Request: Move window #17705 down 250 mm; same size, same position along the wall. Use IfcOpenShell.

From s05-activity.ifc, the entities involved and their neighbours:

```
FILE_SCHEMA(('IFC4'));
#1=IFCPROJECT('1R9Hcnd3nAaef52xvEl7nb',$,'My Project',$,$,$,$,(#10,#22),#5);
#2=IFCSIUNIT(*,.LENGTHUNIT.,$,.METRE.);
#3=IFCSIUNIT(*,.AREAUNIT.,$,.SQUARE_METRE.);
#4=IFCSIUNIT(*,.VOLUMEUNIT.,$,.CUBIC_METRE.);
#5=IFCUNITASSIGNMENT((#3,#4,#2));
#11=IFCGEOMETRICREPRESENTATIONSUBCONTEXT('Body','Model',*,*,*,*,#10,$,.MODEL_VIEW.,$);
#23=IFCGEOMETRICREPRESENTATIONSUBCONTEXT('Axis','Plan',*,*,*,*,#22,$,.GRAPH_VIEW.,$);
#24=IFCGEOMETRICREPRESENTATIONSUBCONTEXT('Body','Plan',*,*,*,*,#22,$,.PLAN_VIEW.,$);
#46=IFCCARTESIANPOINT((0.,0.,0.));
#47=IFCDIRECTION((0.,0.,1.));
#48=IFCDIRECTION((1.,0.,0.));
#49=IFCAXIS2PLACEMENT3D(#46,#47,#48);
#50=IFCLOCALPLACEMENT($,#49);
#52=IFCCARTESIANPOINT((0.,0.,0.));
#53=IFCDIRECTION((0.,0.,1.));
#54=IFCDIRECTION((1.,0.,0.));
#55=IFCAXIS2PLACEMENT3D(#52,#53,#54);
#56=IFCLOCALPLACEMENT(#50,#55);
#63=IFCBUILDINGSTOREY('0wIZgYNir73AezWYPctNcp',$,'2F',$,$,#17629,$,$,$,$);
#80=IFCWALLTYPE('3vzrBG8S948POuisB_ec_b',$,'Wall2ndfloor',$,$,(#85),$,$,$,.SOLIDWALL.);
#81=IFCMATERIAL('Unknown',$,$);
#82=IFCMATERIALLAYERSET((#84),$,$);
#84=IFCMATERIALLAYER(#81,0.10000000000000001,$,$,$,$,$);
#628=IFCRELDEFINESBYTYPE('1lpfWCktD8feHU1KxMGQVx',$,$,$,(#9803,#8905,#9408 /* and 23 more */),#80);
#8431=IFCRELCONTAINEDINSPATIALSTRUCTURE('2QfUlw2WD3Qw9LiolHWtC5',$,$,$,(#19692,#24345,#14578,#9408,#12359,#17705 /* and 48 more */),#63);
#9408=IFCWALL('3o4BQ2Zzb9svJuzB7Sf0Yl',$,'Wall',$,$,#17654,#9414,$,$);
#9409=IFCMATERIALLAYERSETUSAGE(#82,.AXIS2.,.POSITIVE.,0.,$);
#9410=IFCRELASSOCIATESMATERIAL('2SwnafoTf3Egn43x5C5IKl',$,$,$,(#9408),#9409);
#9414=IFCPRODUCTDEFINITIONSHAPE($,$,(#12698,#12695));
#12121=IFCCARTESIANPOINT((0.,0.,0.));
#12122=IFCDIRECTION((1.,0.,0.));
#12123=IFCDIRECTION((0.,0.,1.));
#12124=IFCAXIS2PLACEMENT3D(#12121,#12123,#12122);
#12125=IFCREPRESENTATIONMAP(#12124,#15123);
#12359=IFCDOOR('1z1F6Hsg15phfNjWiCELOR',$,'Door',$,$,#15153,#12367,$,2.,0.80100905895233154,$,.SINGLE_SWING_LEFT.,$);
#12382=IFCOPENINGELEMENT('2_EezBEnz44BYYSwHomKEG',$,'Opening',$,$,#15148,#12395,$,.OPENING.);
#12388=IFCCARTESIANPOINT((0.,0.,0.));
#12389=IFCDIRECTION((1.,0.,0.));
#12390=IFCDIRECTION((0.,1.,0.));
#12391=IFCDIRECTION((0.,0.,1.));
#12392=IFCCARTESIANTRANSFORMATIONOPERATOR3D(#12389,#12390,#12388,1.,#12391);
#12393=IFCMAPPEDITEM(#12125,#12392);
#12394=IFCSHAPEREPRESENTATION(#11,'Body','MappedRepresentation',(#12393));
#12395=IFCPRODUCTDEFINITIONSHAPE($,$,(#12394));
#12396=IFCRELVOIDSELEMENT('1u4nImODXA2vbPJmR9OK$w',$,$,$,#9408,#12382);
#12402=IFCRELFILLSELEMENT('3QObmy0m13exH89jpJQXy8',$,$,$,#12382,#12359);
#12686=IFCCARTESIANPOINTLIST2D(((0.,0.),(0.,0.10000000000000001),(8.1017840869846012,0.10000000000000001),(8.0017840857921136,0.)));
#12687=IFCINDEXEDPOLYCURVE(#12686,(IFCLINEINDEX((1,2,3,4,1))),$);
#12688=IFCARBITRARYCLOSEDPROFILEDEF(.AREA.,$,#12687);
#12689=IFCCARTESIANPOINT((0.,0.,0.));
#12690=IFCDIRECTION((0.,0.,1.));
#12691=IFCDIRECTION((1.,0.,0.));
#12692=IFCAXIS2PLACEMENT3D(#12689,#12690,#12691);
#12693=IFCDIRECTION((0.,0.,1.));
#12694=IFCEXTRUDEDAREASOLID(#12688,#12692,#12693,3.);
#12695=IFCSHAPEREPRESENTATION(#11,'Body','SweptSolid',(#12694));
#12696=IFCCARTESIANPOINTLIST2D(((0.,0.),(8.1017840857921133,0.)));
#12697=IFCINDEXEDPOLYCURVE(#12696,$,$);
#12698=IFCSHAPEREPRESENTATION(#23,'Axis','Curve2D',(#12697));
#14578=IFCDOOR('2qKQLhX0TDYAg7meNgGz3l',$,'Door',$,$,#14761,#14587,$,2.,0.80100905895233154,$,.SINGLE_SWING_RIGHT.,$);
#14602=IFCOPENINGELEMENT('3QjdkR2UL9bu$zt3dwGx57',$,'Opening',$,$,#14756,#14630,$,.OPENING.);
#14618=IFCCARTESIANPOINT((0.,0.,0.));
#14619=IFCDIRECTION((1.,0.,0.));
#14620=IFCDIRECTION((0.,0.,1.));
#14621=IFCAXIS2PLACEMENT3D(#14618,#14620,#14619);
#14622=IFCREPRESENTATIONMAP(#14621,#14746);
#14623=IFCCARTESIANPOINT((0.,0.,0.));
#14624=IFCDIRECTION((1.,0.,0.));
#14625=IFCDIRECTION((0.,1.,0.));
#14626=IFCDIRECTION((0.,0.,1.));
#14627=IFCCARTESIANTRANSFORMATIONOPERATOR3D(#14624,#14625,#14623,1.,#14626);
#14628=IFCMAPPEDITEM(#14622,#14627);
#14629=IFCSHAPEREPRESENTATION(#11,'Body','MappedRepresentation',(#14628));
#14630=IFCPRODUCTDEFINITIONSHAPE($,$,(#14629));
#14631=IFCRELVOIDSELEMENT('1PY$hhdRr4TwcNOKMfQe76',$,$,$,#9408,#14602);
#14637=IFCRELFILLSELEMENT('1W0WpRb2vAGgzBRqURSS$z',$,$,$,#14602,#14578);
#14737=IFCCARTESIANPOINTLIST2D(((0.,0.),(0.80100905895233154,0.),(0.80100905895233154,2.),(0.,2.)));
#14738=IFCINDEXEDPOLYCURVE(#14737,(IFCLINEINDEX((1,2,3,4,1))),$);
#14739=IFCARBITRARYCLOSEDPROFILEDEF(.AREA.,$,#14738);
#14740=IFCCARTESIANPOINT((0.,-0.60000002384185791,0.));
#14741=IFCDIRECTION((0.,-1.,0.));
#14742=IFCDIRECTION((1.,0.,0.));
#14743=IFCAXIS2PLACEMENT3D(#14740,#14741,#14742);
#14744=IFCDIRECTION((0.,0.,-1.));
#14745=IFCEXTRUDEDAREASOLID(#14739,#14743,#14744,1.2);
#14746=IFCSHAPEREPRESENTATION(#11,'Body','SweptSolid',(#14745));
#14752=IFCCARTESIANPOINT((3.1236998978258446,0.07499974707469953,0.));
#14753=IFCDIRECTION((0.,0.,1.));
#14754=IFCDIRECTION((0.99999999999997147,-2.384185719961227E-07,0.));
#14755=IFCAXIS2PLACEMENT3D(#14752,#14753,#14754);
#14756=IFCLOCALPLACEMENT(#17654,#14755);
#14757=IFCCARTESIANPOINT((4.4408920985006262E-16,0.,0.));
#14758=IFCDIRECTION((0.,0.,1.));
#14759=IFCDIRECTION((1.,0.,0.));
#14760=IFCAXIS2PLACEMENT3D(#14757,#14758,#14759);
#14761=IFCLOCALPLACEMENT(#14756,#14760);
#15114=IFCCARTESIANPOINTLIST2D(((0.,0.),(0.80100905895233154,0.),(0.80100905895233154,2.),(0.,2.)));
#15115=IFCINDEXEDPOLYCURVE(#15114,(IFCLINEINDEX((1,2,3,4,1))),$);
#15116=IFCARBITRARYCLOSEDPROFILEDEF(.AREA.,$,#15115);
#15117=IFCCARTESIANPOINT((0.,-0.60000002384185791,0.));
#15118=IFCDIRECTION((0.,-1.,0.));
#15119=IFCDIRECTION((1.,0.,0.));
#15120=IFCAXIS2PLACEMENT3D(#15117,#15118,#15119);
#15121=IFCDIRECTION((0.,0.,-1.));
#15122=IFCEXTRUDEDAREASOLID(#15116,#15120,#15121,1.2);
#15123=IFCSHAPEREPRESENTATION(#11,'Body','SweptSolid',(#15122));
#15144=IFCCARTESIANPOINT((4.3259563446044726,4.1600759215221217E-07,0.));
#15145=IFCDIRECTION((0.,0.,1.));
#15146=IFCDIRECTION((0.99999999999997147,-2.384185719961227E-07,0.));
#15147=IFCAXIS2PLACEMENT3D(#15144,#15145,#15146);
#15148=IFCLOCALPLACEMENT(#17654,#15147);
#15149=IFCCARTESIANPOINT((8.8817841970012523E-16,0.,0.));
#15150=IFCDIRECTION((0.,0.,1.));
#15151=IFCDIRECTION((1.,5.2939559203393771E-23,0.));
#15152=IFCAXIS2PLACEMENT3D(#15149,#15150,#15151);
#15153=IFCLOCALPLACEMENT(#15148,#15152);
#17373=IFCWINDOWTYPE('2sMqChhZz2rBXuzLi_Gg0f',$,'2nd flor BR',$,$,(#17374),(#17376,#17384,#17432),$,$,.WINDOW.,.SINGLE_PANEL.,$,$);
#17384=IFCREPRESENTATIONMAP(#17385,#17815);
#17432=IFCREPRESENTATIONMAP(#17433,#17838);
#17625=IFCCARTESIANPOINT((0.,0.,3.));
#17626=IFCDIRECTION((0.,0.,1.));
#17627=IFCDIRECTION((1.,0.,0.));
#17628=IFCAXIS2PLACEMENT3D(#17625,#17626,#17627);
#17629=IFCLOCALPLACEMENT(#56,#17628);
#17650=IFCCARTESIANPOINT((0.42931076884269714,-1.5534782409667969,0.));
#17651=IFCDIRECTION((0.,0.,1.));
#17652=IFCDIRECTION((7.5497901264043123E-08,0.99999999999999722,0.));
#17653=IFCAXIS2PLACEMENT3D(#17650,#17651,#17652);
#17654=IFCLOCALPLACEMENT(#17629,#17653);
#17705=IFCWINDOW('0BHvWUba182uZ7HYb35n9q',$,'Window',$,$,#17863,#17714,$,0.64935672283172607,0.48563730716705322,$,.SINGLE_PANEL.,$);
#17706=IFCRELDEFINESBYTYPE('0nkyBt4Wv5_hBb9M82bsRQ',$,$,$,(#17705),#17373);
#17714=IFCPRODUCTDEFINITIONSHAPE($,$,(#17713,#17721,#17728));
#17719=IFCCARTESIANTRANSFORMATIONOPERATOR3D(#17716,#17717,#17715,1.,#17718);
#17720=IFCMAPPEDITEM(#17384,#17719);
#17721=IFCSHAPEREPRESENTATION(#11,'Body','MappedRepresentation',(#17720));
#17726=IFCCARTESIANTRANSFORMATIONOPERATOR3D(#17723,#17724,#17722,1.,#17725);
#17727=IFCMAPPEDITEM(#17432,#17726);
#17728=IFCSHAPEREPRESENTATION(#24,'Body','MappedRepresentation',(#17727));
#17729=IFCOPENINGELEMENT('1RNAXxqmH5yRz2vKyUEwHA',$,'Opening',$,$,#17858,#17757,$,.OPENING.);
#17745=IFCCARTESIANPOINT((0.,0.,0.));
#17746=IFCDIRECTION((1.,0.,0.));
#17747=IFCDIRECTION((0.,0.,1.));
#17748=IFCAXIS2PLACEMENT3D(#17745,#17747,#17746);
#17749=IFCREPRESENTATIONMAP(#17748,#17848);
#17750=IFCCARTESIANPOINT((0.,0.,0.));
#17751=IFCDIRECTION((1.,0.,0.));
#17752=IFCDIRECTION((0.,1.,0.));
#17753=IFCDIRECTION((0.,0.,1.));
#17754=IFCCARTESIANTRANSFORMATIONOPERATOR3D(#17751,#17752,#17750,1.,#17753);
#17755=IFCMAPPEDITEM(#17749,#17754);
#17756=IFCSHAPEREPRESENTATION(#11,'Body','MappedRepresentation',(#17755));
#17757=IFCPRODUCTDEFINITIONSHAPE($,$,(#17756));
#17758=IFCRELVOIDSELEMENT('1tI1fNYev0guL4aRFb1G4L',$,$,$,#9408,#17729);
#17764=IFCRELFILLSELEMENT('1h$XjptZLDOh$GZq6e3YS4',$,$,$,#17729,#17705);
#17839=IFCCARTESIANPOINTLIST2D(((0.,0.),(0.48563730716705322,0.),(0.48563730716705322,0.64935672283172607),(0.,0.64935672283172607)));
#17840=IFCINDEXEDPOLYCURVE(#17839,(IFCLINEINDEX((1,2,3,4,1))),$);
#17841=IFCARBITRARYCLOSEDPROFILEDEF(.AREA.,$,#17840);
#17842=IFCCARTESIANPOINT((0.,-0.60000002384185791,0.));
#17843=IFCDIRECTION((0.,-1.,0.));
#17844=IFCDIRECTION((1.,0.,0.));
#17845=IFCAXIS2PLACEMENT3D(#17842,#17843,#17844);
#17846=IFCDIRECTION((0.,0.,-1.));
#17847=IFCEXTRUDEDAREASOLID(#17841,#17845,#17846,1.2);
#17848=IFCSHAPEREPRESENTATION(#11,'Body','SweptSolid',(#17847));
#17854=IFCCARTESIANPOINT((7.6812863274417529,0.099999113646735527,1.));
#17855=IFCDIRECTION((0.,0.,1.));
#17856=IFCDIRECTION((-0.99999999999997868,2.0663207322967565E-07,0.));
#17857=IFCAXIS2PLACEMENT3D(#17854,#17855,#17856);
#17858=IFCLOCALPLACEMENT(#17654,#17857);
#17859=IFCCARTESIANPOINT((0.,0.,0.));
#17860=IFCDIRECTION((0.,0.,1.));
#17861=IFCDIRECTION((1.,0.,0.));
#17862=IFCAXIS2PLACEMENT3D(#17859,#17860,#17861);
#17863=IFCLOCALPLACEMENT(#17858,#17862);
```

```python
import numpy as np
import ifcopenshell
import ifcopenshell.api.geometry
import ifcopenshell.util.placement
import ifcopenshell.util.unit

model = ifcopenshell.open("s05-activity.ifc")
unit_scale = ifcopenshell.util.unit.calculate_unit_scale(model)

window = model.by_id(17705)
opening = window.FillsVoids[0].RelatingOpeningElement
dz = -0.25 / unit_scale

shift = np.array([0.0, 0.0, dz])
# The window is placed relative to its opening, so it follows when the opening moves.
matrix = ifcopenshell.util.placement.get_local_placement(opening.ObjectPlacement)
matrix[:3, 3] += shift
ifcopenshell.api.geometry.edit_object_placement(
    model, product=opening, matrix=matrix, is_si=False, should_transform_children=True
)

print(f"moved by {dz * unit_scale:+.3f} m")

model.write("s05-activity_edited.ifc")
```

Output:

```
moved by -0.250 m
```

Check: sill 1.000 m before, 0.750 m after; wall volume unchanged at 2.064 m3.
